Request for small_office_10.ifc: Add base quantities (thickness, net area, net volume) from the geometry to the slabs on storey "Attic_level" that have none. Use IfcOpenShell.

First a look at what the model holds.

```python
import ifcopenshell
import ifcopenshell.util.element
import ifcopenshell.util.unit

model = ifcopenshell.open("small_office_10.ifc")
print(model.schema)
for unit_type in ("LENGTHUNIT", "AREAUNIT", "VOLUMEUNIT"):
    print(unit_type, ifcopenshell.util.unit.calculate_unit_scale(model, unit_type))
storey = next(s for s in model.by_type("IfcBuildingStorey") if s.Name == "Attic_level")
slabs = [e for e in ifcopenshell.util.element.get_decomposition(storey) if e.is_a("IfcSlab")]
for e in sorted(slabs, key=lambda e: e.id()):
    print(e.id(), e.is_a(), e.Name, list(ifcopenshell.util.element.get_psets(e, qtos_only=True)), sep=" | ")
```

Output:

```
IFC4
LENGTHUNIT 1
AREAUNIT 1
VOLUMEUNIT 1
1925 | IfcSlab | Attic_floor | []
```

```python
import ifcopenshell
import ifcopenshell.api.pset
import ifcopenshell.geom
import ifcopenshell.util.element
import ifcopenshell.util.shape
import ifcopenshell.util.unit

model = ifcopenshell.open("small_office_10.ifc")
unit_scale = ifcopenshell.util.unit.calculate_unit_scale(model)
area_scale = ifcopenshell.util.unit.calculate_unit_scale(model, "AREAUNIT")
volume_scale = ifcopenshell.util.unit.calculate_unit_scale(model, "VOLUMEUNIT")
settings = ifcopenshell.geom.settings()

storey = next(s for s in model.by_type("IfcBuildingStorey") if s.Name == "Attic_level")
slabs = [e for e in ifcopenshell.util.element.get_decomposition(storey) if e.is_a("IfcSlab")]

for e in sorted(slabs, key=lambda e: e.id()):
    if ifcopenshell.util.element.get_psets(e, qtos_only=True, should_inherit=False):
        continue
    # Geometry comes back in metres, in the element's own axes.
    shape = ifcopenshell.geom.create_shape(settings, e)
    values = {
        "Width": ifcopenshell.util.shape.get_z(shape.geometry) / unit_scale,
        "NetArea": ifcopenshell.util.shape.get_footprint_area(shape.geometry) / area_scale,
        "NetVolume": ifcopenshell.util.shape.get_volume(shape.geometry) / volume_scale,
    }
    qto = ifcopenshell.api.pset.add_qto(model, product=e, name="Qto_SlabBaseQuantities")
    ifcopenshell.api.pset.edit_qto(model, qto=qto, properties=values)
    print(e.id(), {k: round(v, 3) for k, v in values.items()})

model.write("small_office_10-out.ifc")
```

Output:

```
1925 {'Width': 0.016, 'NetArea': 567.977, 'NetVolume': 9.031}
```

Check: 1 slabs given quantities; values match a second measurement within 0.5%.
